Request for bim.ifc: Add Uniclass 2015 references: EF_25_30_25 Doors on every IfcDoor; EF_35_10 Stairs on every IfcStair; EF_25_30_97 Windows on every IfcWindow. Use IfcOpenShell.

First a look at what the model holds.

```python
import ifcopenshell

model = ifcopenshell.open("bim.ifc")
print(model.schema)
print("classifications:", [c.Name for c in model.by_type("IfcClassification")])
for ifc_class in ("IfcDoor", "IfcRoof", "IfcStair", "IfcWall", "IfcWindow"):
    print(ifc_class, len(model.by_type(ifc_class)))
```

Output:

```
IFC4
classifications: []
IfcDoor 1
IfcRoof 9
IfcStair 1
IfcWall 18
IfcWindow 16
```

```python
import ifcopenshell
import ifcopenshell.api.classification

model = ifcopenshell.open("bim.ifc")

system = ifcopenshell.api.classification.add_classification(model, classification="Uniclass 2015")

codes = {
    "IfcDoor": ("EF_25_30_25", "Doors"),
    "IfcStair": ("EF_35_10", "Stairs"),
    "IfcWindow": ("EF_25_30_97", "Windows"),
}
for ifc_class, (code, name) in codes.items():
    products = model.by_type(ifc_class)
    ifcopenshell.api.classification.add_reference(
        model, products=products, classification=system, identification=code, name=name
    )
    print(code, len(products))

model.write("bim_rev.ifc")
```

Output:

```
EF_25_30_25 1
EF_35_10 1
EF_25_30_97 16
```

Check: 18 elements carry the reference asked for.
